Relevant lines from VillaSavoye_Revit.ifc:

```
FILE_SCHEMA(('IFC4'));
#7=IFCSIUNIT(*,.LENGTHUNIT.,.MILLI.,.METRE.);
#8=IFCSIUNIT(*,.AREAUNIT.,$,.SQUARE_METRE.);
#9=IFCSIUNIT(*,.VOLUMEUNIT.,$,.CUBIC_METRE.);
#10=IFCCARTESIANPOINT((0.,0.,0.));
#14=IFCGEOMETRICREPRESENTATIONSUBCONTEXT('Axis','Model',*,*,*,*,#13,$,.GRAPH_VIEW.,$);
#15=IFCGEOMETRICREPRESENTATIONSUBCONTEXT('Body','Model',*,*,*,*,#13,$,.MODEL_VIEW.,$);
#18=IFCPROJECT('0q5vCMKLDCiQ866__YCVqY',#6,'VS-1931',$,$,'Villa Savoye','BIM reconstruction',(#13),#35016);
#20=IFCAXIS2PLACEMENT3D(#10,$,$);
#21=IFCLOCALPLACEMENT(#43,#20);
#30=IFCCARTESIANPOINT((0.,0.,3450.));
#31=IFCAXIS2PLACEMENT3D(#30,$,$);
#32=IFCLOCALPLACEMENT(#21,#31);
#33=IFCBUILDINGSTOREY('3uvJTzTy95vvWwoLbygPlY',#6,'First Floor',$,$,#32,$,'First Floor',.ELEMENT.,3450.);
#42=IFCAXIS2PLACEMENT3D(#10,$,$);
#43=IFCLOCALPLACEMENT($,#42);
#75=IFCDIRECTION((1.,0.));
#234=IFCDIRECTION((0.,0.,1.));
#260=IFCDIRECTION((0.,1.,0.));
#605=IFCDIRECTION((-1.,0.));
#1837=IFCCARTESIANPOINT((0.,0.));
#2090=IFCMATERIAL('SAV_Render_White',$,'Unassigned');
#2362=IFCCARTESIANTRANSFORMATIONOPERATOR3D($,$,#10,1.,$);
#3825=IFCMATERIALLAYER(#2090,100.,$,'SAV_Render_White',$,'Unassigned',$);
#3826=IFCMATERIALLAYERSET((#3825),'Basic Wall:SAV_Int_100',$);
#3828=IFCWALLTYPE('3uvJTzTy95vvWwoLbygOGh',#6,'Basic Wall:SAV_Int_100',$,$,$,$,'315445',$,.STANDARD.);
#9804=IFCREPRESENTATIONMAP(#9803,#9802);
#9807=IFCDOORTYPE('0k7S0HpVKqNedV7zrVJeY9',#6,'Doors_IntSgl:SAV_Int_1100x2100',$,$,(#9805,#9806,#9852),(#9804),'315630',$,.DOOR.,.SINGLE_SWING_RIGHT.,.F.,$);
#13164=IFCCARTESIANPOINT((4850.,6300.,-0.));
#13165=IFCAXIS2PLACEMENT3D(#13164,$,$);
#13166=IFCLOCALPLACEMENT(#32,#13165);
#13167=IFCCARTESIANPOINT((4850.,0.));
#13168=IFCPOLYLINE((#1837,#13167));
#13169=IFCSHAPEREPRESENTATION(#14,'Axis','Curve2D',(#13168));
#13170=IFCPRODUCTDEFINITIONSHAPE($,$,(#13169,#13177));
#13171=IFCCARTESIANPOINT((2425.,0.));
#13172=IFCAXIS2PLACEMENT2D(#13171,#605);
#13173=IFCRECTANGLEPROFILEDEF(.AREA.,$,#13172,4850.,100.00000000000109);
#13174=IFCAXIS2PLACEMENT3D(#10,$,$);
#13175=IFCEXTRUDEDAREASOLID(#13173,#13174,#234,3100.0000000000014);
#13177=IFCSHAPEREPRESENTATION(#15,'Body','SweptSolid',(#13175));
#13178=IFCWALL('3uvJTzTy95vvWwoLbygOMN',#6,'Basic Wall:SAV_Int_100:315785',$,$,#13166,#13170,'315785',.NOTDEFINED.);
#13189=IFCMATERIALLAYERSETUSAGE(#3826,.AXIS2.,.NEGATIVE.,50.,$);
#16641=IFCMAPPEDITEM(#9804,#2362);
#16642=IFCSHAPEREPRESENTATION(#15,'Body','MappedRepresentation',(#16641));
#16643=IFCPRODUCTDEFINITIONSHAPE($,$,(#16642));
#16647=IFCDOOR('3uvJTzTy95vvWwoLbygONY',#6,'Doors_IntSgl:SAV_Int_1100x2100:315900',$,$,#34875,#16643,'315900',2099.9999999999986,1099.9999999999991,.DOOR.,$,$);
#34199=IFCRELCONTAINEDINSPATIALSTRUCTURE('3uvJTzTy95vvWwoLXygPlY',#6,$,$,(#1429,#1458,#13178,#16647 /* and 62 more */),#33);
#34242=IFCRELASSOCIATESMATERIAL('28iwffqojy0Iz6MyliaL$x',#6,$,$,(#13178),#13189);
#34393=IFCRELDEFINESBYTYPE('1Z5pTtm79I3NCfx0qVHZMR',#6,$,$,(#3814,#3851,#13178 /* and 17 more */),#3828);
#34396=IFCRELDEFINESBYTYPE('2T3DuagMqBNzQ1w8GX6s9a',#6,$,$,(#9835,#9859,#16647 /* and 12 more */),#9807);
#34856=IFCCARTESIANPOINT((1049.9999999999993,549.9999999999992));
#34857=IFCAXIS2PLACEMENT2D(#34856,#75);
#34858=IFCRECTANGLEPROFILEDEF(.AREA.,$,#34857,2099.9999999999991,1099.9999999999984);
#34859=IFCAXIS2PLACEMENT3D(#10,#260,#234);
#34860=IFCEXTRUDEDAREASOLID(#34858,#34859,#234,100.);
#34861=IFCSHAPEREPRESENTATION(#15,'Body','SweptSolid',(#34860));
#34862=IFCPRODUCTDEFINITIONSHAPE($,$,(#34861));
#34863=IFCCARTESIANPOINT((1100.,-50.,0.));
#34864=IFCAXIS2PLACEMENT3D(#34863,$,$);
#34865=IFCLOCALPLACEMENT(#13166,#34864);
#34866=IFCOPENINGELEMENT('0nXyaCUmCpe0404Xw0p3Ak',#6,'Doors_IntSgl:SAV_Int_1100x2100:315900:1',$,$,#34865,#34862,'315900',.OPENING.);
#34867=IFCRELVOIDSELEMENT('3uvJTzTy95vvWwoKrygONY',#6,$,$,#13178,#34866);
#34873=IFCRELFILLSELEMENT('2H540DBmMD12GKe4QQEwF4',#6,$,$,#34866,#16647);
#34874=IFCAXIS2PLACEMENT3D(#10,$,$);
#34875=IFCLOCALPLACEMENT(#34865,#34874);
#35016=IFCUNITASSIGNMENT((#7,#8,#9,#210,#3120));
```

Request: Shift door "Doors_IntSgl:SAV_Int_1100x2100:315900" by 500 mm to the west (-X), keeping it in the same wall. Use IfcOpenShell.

```python
import ifcopenshell
import ifcopenshell.api.geometry
import ifcopenshell.util.placement
import ifcopenshell.util.unit

model = ifcopenshell.open("VillaSavoye_Revit.ifc")
unit_scale = ifcopenshell.util.unit.calculate_unit_scale(model)

door = model.by_guid("3uvJTzTy95vvWwoLbygONY")
opening = door.FillsVoids[0].RelatingOpeningElement
wall = opening.VoidsElements[0].RelatingBuildingElement

wall_matrix = ifcopenshell.util.placement.get_local_placement(wall.ObjectPlacement)
shift = wall_matrix[:3, 0] * -0.5 / unit_scale
before = ifcopenshell.util.placement.get_local_placement(door.ObjectPlacement)[:3, 3].copy()

# The door is placed relative to its opening, so it follows when the opening moves.
matrix = ifcopenshell.util.placement.get_local_placement(opening.ObjectPlacement)
matrix[:3, 3] += shift
ifcopenshell.api.geometry.edit_object_placement(
    model, product=opening, matrix=matrix, is_si=False, should_transform_children=True
)

after = ifcopenshell.util.placement.get_local_placement(door.ObjectPlacement)[:3, 3]
print("door moved by", (after - before).round(3) + 0.0)

model.write("VillaSavoye_Revit_edited.ifc")
```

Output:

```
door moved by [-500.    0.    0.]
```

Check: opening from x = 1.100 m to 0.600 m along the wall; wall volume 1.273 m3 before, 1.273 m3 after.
